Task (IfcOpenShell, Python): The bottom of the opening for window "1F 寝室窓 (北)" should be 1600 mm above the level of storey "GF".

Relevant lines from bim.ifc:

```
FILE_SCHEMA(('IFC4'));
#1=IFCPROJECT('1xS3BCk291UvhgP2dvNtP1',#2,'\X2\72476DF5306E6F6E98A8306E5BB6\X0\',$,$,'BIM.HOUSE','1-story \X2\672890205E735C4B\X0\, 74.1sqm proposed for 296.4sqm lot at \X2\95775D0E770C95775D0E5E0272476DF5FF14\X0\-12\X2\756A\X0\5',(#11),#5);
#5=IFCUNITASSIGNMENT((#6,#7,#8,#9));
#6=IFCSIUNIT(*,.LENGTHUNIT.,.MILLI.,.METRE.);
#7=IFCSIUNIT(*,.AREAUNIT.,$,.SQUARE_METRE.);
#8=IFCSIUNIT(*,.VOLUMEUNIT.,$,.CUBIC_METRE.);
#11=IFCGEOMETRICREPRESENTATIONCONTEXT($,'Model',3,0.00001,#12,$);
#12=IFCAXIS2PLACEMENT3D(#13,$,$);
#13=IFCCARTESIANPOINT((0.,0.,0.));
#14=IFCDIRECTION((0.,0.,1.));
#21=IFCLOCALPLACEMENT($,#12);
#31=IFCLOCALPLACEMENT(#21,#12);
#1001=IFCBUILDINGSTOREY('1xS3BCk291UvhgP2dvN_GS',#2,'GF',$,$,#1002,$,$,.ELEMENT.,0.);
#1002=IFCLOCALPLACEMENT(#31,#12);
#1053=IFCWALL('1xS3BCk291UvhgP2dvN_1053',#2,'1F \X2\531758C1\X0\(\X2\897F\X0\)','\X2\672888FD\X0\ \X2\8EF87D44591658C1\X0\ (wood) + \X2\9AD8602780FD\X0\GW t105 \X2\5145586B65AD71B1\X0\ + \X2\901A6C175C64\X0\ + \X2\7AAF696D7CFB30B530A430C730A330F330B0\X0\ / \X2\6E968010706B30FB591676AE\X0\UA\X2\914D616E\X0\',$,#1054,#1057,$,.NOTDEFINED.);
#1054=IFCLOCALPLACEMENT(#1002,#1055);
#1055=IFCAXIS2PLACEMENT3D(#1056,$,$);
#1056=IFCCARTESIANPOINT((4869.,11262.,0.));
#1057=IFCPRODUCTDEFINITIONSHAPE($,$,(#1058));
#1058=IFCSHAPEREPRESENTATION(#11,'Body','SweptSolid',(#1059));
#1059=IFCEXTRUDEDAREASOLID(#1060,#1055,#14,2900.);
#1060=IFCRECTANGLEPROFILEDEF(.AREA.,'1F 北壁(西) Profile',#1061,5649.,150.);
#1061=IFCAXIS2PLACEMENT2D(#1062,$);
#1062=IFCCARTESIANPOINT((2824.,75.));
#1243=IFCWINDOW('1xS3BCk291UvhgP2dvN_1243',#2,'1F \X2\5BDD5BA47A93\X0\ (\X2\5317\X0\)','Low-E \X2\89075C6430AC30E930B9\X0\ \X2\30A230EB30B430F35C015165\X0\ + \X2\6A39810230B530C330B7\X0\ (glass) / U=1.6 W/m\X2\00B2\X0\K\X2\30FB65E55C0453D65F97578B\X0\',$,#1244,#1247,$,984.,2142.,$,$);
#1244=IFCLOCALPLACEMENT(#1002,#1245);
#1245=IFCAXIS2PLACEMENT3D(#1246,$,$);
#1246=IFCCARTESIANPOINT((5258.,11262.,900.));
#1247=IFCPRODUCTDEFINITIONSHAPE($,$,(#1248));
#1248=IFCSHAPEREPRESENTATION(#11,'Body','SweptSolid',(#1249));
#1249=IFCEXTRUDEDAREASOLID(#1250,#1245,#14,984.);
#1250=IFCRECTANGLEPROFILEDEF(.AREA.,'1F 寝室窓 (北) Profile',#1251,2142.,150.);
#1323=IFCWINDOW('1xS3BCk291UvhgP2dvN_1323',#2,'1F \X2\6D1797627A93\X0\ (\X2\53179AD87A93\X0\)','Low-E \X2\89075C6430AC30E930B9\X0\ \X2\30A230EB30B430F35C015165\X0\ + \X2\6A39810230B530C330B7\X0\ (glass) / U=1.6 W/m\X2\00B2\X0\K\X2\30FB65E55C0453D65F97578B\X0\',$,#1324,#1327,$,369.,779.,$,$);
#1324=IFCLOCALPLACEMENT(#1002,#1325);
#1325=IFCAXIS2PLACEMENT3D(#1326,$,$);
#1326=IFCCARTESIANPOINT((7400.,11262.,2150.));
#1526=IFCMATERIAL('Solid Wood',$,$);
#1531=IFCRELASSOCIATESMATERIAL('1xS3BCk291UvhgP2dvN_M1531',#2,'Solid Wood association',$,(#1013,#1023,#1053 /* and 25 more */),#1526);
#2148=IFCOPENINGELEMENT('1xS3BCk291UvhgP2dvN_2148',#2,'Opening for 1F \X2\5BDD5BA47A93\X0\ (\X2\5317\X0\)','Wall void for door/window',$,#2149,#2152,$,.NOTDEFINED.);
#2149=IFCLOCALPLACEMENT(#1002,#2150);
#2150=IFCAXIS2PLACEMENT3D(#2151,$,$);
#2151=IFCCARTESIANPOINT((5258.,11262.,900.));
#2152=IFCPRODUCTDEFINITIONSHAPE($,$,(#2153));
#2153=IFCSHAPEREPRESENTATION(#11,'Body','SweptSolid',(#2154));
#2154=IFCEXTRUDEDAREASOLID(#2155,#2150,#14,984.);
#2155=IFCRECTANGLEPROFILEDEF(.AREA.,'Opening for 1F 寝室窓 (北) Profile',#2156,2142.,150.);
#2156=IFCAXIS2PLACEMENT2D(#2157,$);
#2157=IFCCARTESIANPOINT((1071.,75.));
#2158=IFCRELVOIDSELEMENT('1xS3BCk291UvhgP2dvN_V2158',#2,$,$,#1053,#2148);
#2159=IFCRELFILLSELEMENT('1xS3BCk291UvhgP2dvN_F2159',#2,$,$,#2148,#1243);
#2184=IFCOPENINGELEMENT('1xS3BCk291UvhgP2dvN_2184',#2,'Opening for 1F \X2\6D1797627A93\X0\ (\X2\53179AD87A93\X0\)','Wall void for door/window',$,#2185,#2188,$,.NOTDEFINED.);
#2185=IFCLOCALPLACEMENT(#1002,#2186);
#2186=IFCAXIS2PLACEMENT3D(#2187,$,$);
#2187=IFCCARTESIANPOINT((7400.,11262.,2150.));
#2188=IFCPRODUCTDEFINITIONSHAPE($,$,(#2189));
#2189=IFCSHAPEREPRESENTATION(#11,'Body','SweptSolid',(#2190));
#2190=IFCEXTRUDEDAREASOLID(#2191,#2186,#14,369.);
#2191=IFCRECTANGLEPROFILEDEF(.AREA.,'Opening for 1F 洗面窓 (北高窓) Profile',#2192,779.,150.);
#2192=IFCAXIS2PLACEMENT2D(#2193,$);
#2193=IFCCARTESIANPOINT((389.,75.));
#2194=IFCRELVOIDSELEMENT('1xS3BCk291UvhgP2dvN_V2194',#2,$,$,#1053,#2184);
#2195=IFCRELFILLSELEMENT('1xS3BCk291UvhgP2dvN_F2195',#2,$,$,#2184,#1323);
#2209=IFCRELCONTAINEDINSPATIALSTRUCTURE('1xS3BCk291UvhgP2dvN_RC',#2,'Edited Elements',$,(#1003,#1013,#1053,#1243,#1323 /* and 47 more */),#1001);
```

```python
import numpy as np
import ifcopenshell
import ifcopenshell.api.geometry
import ifcopenshell.geom
import ifcopenshell.util.element
import ifcopenshell.util.placement
import ifcopenshell.util.shape
import ifcopenshell.util.unit

model = ifcopenshell.open("bim.ifc")
unit_scale = ifcopenshell.util.unit.calculate_unit_scale(model)

window = model.by_guid("1xS3BCk291UvhgP2dvN_1243")
opening = window.FillsVoids[0].RelatingOpeningElement
storey = ifcopenshell.util.element.get_container(window, ifc_class="IfcBuildingStorey")
level = ifcopenshell.util.placement.get_local_placement(storey.ObjectPlacement)[2, 3]

# The opening's origin need not be at the sill, so measure its lowest point.
shape = ifcopenshell.geom.create_shape(ifcopenshell.geom.settings(), opening)
bottom = ifcopenshell.util.shape.get_shape_bottom_elevation(shape, shape.geometry) / unit_scale
dz = level + 1.6 / unit_scale - bottom

shift = np.array([0.0, 0.0, dz])
# The window is not placed relative to its opening, so move both.
for product in (opening, window):
    matrix = ifcopenshell.util.placement.get_local_placement(product.ObjectPlacement)
    matrix[:3, 3] += shift
    ifcopenshell.api.geometry.edit_object_placement(model, product=product, matrix=matrix, is_si=False)

print(f"moved by {dz * unit_scale:+.3f} m")

model.write("bim_rev.ifc")
```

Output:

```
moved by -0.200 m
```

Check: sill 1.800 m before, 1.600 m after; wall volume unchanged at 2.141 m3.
